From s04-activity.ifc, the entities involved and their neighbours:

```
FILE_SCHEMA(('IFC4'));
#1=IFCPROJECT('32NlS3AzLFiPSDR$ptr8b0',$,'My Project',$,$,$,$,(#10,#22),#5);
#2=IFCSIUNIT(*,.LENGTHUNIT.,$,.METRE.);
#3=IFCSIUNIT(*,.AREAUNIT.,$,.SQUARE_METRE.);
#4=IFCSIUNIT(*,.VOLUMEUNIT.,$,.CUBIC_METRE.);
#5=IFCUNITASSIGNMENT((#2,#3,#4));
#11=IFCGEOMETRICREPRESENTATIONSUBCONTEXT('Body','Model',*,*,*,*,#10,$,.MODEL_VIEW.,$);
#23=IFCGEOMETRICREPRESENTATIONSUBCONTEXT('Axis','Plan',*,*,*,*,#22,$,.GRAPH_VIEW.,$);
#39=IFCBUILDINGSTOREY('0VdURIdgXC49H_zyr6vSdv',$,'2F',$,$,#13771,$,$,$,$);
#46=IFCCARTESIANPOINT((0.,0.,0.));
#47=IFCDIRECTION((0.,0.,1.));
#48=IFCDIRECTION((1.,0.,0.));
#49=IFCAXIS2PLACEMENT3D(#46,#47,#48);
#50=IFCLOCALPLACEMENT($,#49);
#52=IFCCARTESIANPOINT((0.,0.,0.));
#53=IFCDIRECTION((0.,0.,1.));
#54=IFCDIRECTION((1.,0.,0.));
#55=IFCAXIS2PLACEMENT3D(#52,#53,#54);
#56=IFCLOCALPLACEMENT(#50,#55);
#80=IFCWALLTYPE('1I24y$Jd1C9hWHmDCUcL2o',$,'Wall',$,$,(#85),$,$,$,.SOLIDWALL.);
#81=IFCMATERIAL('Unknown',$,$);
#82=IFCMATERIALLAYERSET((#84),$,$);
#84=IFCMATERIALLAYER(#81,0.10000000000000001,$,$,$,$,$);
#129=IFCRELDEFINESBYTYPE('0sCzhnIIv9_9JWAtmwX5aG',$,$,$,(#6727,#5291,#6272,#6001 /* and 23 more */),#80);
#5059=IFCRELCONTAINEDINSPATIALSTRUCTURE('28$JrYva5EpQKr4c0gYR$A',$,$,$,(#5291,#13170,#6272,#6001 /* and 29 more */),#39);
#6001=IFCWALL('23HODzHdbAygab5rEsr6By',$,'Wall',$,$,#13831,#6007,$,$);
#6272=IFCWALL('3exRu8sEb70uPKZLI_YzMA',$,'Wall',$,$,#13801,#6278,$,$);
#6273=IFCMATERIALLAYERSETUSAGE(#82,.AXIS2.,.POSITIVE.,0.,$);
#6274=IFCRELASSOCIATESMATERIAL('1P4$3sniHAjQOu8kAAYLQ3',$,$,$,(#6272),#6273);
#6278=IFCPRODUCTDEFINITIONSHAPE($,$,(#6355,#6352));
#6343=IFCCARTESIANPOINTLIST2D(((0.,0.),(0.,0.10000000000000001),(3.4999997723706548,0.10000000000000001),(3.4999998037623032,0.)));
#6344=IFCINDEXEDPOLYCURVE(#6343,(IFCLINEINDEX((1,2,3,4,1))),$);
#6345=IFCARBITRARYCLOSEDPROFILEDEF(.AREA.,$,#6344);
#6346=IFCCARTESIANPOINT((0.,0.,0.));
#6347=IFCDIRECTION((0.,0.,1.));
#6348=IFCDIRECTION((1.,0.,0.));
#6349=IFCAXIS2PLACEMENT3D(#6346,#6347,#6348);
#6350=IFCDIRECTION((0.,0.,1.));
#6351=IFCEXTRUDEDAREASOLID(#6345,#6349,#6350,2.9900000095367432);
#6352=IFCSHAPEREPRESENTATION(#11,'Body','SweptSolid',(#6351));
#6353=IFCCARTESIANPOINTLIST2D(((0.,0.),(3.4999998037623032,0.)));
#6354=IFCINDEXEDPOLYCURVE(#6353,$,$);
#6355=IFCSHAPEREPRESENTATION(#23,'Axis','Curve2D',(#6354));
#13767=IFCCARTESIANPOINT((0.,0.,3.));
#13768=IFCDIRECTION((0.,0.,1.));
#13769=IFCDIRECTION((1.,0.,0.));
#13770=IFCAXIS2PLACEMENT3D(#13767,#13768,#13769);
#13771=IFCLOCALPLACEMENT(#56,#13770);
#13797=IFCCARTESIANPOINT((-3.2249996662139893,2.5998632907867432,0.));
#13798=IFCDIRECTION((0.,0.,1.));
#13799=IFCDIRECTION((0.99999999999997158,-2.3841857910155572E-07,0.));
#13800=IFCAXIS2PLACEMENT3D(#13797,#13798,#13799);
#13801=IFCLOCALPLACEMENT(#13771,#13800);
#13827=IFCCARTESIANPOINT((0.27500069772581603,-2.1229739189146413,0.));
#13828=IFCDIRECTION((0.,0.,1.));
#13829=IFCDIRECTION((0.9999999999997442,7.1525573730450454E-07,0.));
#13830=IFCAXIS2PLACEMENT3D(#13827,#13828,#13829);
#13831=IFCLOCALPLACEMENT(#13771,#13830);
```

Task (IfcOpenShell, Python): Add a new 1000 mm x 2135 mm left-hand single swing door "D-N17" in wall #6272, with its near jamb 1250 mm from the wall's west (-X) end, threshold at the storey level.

```python
import numpy as np
import ifcopenshell
import ifcopenshell.api.feature
import ifcopenshell.api.geometry
import ifcopenshell.api.root
import ifcopenshell.api.spatial
import ifcopenshell.geom
import ifcopenshell.util.element
import ifcopenshell.util.placement
import ifcopenshell.util.representation
import ifcopenshell.util.shape
import ifcopenshell.util.unit

model = ifcopenshell.open("s04-activity.ifc")
unit_scale = ifcopenshell.util.unit.calculate_unit_scale(model)
settings = ifcopenshell.geom.settings()


def volume(element):
    """Net volume in cubic metres, openings subtracted."""
    shape = ifcopenshell.geom.create_shape(settings, element)
    return ifcopenshell.util.shape.get_volume(shape.geometry)


wall = model.by_guid("3exRu8sEb70uPKZLI_YzMA")
storey = ifcopenshell.util.element.get_container(wall, ifc_class="IfcBuildingStorey")
context = ifcopenshell.util.representation.get_context(model, "Model", "Body", "MODEL_VIEW")
before = volume(wall)

width, height, from_end, sill = 1, 2.135, 1.25, 0.0  # metres

# The wall runs along its own X axis, and the end named is its -X end.
wall_shape = ifcopenshell.geom.create_shape(settings, wall)
x, y, z = ifcopenshell.util.shape.get_vertices(wall_shape.geometry).T
start = x.min() + from_end
face, thickness = float(y.min()), float(y.max() - y.min())
wall_matrix = ifcopenshell.util.placement.get_local_placement(wall.ObjectPlacement)
level = ifcopenshell.util.placement.get_local_placement(storey.ObjectPlacement)[2, 3]


def in_wall(x, y):
    """Placement at x, y metres in the wall's axes, at sill height."""
    matrix = wall_matrix.copy()
    matrix[:, 3] = wall_matrix @ np.array([x / unit_scale, y / unit_scale, 0.0, 1.0])
    matrix[2, 3] = level + sill / unit_scale
    return matrix


# Opening: a box that overshoots both wall faces by 50 mm.
opening = ifcopenshell.api.root.create_entity(model, ifc_class="IfcOpeningElement", predefined_type="OPENING")
box = ifcopenshell.api.geometry.add_wall_representation(
    model, context=context, length=width, height=height, thickness=thickness + 0.1
)
ifcopenshell.api.geometry.assign_representation(model, product=opening, representation=box)
ifcopenshell.api.geometry.edit_object_placement(model, product=opening, matrix=in_wall(start, face - 0.05), is_si=False)
ifcopenshell.api.feature.add_feature(model, feature=opening, element=wall)

door = ifcopenshell.api.root.create_entity(model, ifc_class="IfcDoor", name="D-N17", predefined_type="DOOR")
door.OverallWidth, door.OverallHeight = width / unit_scale, height / unit_scale
door.OperationType = "SINGLE_SWING_LEFT"
body = ifcopenshell.api.geometry.add_door_representation(
    model,
    context=context,
    overall_width=door.OverallWidth,
    overall_height=door.OverallHeight,
    operation_type="SINGLE_SWING_LEFT",
    lining_properties={"LiningDepth": thickness / unit_scale, "ThresholdDepth": thickness / unit_scale},
)
ifcopenshell.api.geometry.assign_representation(model, product=door, representation=body)
ifcopenshell.api.spatial.assign_container(model, products=[door], relating_structure=storey)
ifcopenshell.api.feature.add_filling(model, opening=opening, element=door)

# The lining spans the wall, so the door starts at the wall face.
ifcopenshell.api.geometry.edit_object_placement(model, product=door, matrix=in_wall(start, face), is_si=False)

after = volume(wall)

print(f"wall volume {before:.3f} -> {after:.3f} m3")

model.write("s04-activity-out.ifc")
```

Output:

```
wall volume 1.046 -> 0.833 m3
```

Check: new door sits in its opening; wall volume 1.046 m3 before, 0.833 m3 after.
